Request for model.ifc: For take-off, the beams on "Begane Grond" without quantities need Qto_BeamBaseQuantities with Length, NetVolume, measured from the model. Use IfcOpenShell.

First a look at what the model holds.

```python
import ifcopenshell
import ifcopenshell.util.element
import ifcopenshell.util.unit

model = ifcopenshell.open("model.ifc")
print(model.schema)
for unit_type in ("LENGTHUNIT", "AREAUNIT", "VOLUMEUNIT"):
    print(unit_type, ifcopenshell.util.unit.calculate_unit_scale(model, unit_type))
storey = next(s for s in model.by_type("IfcBuildingStorey") if s.Name == "Begane Grond")
beams = [e for e in ifcopenshell.util.element.get_decomposition(storey) if e.is_a("IfcBeam")]
for e in sorted(beams, key=lambda e: e.id()):
    print(e.id(), e.is_a(), e.Name, list(ifcopenshell.util.element.get_psets(e, qtos_only=True)), sep=" | ")
```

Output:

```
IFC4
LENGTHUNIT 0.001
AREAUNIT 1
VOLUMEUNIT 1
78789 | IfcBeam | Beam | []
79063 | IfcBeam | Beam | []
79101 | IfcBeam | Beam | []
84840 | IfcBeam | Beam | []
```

```python
import ifcopenshell
import ifcopenshell.api.pset
import ifcopenshell.geom
import ifcopenshell.util.element
import ifcopenshell.util.shape
import ifcopenshell.util.unit

model = ifcopenshell.open("model.ifc")
unit_scale = ifcopenshell.util.unit.calculate_unit_scale(model)
volume_scale = ifcopenshell.util.unit.calculate_unit_scale(model, "VOLUMEUNIT")
settings = ifcopenshell.geom.settings()

storey = next(s for s in model.by_type("IfcBuildingStorey") if s.Name == "Begane Grond")
beams = [e for e in ifcopenshell.util.element.get_decomposition(storey) if e.is_a("IfcBeam")]

for e in sorted(beams, key=lambda e: e.id()):
    if ifcopenshell.util.element.get_psets(e, qtos_only=True, should_inherit=False):
        continue
    # Geometry comes back in metres, in the element's own axes.
    shape = ifcopenshell.geom.create_shape(settings, e)
    values = {
        "Length": ifcopenshell.util.shape.get_max_xyz(shape.geometry) / unit_scale,
        "NetVolume": ifcopenshell.util.shape.get_volume(shape.geometry) / volume_scale,
    }
    qto = ifcopenshell.api.pset.add_qto(model, product=e, name="Qto_BeamBaseQuantities")
    ifcopenshell.api.pset.edit_qto(model, qto=qto, properties=values)
    print(e.id(), {k: round(v, 3) for k, v in values.items()})

model.write("model-out.ifc")
```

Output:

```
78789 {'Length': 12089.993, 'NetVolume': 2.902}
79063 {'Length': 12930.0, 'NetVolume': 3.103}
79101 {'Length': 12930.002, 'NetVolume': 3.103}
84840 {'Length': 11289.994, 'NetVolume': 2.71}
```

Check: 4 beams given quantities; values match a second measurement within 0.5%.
